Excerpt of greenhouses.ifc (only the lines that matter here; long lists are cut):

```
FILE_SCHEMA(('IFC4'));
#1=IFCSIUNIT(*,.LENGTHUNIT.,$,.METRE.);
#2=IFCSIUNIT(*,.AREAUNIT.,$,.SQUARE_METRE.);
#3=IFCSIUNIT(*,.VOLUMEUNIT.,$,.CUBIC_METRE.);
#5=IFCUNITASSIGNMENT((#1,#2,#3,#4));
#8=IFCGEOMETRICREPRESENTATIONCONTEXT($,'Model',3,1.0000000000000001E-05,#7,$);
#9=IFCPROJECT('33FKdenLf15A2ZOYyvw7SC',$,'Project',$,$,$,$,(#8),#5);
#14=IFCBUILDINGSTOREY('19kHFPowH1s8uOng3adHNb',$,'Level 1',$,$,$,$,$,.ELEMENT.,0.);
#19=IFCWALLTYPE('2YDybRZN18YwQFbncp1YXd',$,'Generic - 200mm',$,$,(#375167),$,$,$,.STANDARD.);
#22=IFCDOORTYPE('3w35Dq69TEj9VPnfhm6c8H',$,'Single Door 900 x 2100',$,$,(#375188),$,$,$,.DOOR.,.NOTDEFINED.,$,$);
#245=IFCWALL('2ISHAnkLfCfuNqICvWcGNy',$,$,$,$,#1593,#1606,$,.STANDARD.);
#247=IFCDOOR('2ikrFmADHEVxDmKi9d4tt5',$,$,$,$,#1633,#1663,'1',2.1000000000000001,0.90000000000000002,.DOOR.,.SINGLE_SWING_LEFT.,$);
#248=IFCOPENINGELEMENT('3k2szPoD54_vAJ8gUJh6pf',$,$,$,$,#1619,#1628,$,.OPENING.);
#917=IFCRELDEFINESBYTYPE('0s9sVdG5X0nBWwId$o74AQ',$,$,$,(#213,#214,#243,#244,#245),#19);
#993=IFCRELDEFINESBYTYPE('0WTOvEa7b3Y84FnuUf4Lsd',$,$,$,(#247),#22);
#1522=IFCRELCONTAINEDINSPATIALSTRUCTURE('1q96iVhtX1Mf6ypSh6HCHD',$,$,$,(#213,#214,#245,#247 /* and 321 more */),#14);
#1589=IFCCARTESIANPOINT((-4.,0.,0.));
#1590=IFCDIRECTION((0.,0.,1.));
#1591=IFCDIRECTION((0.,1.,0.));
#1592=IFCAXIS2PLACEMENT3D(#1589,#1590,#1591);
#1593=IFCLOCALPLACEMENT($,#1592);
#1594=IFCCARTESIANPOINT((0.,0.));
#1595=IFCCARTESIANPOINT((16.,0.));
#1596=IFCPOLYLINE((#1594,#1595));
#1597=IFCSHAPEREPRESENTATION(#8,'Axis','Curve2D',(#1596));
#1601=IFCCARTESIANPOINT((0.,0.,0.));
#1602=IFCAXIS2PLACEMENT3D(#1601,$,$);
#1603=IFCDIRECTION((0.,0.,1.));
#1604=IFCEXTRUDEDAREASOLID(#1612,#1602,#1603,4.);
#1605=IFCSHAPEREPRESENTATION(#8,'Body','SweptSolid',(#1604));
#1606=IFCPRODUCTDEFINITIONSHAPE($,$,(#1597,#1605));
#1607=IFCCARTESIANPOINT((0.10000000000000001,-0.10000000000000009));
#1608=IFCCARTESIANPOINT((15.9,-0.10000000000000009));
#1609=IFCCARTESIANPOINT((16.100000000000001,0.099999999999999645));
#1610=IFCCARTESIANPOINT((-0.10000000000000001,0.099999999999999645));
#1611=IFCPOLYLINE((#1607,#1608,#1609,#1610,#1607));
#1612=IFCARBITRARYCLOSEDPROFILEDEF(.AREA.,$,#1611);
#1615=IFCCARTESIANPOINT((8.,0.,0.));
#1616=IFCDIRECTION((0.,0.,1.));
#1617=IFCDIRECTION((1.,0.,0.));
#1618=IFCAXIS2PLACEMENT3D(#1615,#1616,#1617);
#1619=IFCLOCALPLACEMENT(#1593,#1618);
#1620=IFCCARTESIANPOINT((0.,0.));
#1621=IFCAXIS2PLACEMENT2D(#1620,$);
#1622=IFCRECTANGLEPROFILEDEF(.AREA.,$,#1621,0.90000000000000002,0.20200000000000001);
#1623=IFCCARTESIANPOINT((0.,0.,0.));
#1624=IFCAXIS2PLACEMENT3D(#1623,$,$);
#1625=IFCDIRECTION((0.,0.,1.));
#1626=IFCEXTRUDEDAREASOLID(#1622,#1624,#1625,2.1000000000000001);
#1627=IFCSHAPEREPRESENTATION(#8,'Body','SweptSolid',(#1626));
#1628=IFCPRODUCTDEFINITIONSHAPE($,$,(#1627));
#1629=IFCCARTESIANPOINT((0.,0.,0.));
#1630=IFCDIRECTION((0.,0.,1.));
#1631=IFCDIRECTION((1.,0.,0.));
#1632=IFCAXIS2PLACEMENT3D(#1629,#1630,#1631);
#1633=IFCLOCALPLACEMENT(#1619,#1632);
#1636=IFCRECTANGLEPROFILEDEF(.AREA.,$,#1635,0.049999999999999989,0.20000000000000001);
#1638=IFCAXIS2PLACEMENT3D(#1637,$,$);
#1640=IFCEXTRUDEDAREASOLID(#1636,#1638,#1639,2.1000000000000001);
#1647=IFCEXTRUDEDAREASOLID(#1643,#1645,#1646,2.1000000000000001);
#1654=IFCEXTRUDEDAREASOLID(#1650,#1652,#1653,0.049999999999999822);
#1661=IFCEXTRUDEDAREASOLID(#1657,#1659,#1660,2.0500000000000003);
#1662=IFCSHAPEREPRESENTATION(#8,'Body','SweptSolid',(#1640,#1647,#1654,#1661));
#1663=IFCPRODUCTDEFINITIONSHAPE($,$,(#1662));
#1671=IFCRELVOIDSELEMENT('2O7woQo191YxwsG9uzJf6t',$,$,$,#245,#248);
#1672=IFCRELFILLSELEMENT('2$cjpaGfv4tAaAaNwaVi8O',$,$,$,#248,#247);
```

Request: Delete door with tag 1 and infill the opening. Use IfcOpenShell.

```python
import ifcopenshell
import ifcopenshell.api.feature
import ifcopenshell.api.root
import ifcopenshell.geom
import ifcopenshell.util.shape

model = ifcopenshell.open("greenhouses.ifc")
settings = ifcopenshell.geom.settings()


def volume(element):
    """Net volume in cubic metres, openings subtracted."""
    shape = ifcopenshell.geom.create_shape(settings, element)
    return ifcopenshell.util.shape.get_volume(shape.geometry)


door = model.by_id(247)
opening = door.FillsVoids[0].RelatingOpeningElement
wall = opening.VoidsElements[0].RelatingBuildingElement
before = volume(wall)

ifcopenshell.api.root.remove_product(model, product=door)
ifcopenshell.api.feature.remove_feature(model, feature=opening)

after = volume(wall)

print(f"wall volume {before:.3f} -> {after:.3f} m3")

model.write("greenhouses-out.ifc")
```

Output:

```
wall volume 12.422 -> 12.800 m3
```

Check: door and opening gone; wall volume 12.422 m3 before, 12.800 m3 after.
